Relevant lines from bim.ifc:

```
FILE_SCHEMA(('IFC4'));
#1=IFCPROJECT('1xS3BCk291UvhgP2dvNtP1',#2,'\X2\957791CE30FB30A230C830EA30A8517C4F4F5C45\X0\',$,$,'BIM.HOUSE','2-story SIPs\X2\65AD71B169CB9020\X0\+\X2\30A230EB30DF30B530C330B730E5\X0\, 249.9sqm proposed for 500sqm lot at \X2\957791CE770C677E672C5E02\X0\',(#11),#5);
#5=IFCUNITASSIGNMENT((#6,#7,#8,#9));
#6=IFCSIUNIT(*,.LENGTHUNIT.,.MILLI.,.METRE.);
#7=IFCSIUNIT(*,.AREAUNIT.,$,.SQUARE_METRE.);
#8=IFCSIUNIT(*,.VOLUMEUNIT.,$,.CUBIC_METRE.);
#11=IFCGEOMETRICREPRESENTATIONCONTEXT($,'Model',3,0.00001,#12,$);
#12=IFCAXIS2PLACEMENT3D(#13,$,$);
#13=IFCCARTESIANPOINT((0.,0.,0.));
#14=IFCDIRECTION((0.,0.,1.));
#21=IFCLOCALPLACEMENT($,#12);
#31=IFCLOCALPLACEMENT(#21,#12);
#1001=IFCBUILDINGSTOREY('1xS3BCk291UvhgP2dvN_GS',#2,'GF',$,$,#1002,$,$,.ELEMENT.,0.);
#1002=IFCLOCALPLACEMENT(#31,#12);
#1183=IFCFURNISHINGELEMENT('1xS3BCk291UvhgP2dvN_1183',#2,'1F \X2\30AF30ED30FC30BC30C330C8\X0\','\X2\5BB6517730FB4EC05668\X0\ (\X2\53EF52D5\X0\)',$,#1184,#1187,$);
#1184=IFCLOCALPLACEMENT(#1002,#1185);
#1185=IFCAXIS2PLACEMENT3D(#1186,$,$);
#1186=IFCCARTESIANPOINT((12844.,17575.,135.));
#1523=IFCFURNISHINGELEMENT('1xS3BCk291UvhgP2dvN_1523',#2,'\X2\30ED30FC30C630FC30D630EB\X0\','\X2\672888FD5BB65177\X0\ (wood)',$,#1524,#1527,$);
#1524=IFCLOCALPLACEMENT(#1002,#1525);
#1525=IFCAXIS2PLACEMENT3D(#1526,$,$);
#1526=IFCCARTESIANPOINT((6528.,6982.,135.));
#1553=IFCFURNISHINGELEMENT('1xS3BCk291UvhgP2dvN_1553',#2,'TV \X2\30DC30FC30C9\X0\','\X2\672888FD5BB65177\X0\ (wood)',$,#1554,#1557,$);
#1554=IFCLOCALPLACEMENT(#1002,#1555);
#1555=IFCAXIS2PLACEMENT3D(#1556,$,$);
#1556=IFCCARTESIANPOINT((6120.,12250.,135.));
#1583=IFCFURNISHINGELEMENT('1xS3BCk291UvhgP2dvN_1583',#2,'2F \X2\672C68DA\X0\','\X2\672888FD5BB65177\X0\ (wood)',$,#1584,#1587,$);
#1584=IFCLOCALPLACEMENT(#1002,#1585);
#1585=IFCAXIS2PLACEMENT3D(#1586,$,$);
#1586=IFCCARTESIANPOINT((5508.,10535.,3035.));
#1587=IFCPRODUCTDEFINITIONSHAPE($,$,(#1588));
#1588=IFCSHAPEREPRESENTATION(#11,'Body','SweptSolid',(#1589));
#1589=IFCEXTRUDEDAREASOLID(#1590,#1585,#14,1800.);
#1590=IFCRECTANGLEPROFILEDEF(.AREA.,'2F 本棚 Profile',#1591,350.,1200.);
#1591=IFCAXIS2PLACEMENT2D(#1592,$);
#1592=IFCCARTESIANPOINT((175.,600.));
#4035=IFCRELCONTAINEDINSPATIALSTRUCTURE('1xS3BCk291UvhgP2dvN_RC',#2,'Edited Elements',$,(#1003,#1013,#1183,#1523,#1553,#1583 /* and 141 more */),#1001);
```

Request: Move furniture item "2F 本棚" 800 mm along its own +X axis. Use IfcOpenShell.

```python
import ifcopenshell
import ifcopenshell.api.geometry
import ifcopenshell.util.placement

model = ifcopenshell.open("bim.ifc")

item = model.by_guid("1xS3BCk291UvhgP2dvN_1583")
matrix = ifcopenshell.util.placement.get_local_placement(item.ObjectPlacement)
matrix[:3, 3] += matrix[:3, 0] * 800.0
ifcopenshell.api.geometry.edit_object_placement(model, product=item, matrix=matrix, is_si=False)

print(ifcopenshell.util.placement.get_local_placement(item.ObjectPlacement).round(3) + 0.0)

model.write("bim_edited.ifc")
```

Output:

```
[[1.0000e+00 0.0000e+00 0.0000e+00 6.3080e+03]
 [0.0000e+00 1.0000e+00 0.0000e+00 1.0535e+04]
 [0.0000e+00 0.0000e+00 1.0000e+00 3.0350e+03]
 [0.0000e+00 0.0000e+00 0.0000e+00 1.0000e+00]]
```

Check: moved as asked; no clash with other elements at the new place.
